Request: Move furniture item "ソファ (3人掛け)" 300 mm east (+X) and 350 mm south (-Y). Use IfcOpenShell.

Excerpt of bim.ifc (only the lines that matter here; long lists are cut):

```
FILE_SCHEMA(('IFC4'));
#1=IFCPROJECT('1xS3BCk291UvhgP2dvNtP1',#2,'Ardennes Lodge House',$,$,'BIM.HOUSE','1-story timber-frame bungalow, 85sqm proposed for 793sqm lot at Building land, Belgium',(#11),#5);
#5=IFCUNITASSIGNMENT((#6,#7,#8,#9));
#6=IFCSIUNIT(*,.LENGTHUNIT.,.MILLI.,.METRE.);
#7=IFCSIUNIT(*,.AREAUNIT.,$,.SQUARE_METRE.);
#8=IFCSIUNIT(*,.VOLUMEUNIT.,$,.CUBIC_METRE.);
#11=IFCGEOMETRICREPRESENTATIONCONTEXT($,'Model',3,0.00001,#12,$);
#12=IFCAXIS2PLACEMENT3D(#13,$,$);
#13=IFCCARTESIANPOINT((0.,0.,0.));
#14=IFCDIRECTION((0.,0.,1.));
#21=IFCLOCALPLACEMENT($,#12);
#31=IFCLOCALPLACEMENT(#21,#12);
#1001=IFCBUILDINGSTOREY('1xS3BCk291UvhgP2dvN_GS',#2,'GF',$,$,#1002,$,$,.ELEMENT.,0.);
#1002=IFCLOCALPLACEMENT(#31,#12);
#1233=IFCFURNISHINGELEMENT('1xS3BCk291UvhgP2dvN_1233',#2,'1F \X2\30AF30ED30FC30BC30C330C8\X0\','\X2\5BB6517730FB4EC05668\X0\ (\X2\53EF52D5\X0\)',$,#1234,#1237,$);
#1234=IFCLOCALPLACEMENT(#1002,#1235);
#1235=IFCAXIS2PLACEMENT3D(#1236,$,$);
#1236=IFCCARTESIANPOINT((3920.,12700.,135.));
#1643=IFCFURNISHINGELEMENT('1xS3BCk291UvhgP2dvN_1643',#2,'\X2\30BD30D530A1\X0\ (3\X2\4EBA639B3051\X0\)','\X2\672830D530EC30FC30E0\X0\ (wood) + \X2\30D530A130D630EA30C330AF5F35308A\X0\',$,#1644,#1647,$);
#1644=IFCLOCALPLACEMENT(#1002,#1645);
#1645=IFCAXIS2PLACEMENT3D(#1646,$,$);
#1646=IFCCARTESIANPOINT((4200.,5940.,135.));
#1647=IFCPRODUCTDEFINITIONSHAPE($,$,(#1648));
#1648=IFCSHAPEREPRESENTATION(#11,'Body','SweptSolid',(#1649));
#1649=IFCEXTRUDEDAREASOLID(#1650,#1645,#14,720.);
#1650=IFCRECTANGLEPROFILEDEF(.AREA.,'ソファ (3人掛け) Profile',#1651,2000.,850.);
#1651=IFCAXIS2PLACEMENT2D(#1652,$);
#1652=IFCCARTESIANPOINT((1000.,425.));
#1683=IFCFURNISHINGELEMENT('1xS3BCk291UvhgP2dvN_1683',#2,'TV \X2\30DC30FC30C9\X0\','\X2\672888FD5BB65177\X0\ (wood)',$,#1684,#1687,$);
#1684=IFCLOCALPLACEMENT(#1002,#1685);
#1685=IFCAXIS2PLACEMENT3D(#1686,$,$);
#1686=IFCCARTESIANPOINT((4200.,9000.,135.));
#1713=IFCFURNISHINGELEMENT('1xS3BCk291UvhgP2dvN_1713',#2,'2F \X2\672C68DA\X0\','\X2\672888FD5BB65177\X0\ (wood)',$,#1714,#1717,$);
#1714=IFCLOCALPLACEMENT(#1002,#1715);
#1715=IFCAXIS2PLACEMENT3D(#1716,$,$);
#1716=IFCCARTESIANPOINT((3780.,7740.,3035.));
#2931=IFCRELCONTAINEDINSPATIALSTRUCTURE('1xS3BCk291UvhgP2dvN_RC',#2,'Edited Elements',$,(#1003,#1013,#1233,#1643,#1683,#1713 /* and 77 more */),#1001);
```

```python
import ifcopenshell
import ifcopenshell.api.geometry
import ifcopenshell.util.placement

model = ifcopenshell.open("bim.ifc")

item = model.by_id(1643)
matrix = ifcopenshell.util.placement.get_local_placement(item.ObjectPlacement)
matrix[0, 3] += 300.0
matrix[1, 3] -= 350.0
ifcopenshell.api.geometry.edit_object_placement(model, product=item, matrix=matrix, is_si=False)

print(ifcopenshell.util.placement.get_local_placement(item.ObjectPlacement).round(3) + 0.0)

model.write("bim_v2.ifc")
```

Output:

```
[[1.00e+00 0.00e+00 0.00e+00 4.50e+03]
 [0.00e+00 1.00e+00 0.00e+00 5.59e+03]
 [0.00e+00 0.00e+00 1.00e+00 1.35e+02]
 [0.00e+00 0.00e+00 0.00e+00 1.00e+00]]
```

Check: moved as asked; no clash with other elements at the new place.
